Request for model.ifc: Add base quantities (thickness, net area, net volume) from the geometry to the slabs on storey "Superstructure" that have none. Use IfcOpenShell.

First a look at what the model holds.

```python
import ifcopenshell
import ifcopenshell.util.element
import ifcopenshell.util.unit

model = ifcopenshell.open("model.ifc")
print(model.schema)
for unit_type in ("LENGTHUNIT", "AREAUNIT", "VOLUMEUNIT"):
    print(unit_type, ifcopenshell.util.unit.calculate_unit_scale(model, unit_type))
storey = next(s for s in model.by_type("IfcBuildingStorey") if s.Name == "Superstructure")
slabs = [e for e in ifcopenshell.util.element.get_decomposition(storey) if e.is_a("IfcSlab")]
for e in sorted(slabs, key=lambda e: e.id()):
    print(e.id(), e.is_a(), e.Name, list(ifcopenshell.util.element.get_psets(e, qtos_only=True)), sep=" | ")
```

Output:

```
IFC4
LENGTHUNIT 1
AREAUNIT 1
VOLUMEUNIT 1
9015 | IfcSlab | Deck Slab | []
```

```python
import ifcopenshell
import ifcopenshell.api.pset
import ifcopenshell.geom
import ifcopenshell.util.element
import ifcopenshell.util.shape
import ifcopenshell.util.unit

model = ifcopenshell.open("model.ifc")
unit_scale = ifcopenshell.util.unit.calculate_unit_scale(model)
area_scale = ifcopenshell.util.unit.calculate_unit_scale(model, "AREAUNIT")
volume_scale = ifcopenshell.util.unit.calculate_unit_scale(model, "VOLUMEUNIT")
settings = ifcopenshell.geom.settings()

storey = next(s for s in model.by_type("IfcBuildingStorey") if s.Name == "Superstructure")
slabs = [e for e in ifcopenshell.util.element.get_decomposition(storey) if e.is_a("IfcSlab")]

for e in sorted(slabs, key=lambda e: e.id()):
    if ifcopenshell.util.element.get_psets(e, qtos_only=True, should_inherit=False):
        continue
    # Geometry comes back in metres, in the element's own axes.
    shape = ifcopenshell.geom.create_shape(settings, e)
    values = {
        "Width": ifcopenshell.util.shape.get_z(shape.geometry) / unit_scale,
        "NetArea": ifcopenshell.util.shape.get_footprint_area(shape.geometry) / area_scale,
        "NetVolume": ifcopenshell.util.shape.get_volume(shape.geometry) / volume_scale,
    }
    qto = ifcopenshell.api.pset.add_qto(model, product=e, name="Qto_SlabBaseQuantities")
    ifcopenshell.api.pset.edit_qto(model, qto=qto, properties=values)
    print(e.id(), {k: round(v, 3) for k, v in values.items()})

model.write("model_rev.ifc")
```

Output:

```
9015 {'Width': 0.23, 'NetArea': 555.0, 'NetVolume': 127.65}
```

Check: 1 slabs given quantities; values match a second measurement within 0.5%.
